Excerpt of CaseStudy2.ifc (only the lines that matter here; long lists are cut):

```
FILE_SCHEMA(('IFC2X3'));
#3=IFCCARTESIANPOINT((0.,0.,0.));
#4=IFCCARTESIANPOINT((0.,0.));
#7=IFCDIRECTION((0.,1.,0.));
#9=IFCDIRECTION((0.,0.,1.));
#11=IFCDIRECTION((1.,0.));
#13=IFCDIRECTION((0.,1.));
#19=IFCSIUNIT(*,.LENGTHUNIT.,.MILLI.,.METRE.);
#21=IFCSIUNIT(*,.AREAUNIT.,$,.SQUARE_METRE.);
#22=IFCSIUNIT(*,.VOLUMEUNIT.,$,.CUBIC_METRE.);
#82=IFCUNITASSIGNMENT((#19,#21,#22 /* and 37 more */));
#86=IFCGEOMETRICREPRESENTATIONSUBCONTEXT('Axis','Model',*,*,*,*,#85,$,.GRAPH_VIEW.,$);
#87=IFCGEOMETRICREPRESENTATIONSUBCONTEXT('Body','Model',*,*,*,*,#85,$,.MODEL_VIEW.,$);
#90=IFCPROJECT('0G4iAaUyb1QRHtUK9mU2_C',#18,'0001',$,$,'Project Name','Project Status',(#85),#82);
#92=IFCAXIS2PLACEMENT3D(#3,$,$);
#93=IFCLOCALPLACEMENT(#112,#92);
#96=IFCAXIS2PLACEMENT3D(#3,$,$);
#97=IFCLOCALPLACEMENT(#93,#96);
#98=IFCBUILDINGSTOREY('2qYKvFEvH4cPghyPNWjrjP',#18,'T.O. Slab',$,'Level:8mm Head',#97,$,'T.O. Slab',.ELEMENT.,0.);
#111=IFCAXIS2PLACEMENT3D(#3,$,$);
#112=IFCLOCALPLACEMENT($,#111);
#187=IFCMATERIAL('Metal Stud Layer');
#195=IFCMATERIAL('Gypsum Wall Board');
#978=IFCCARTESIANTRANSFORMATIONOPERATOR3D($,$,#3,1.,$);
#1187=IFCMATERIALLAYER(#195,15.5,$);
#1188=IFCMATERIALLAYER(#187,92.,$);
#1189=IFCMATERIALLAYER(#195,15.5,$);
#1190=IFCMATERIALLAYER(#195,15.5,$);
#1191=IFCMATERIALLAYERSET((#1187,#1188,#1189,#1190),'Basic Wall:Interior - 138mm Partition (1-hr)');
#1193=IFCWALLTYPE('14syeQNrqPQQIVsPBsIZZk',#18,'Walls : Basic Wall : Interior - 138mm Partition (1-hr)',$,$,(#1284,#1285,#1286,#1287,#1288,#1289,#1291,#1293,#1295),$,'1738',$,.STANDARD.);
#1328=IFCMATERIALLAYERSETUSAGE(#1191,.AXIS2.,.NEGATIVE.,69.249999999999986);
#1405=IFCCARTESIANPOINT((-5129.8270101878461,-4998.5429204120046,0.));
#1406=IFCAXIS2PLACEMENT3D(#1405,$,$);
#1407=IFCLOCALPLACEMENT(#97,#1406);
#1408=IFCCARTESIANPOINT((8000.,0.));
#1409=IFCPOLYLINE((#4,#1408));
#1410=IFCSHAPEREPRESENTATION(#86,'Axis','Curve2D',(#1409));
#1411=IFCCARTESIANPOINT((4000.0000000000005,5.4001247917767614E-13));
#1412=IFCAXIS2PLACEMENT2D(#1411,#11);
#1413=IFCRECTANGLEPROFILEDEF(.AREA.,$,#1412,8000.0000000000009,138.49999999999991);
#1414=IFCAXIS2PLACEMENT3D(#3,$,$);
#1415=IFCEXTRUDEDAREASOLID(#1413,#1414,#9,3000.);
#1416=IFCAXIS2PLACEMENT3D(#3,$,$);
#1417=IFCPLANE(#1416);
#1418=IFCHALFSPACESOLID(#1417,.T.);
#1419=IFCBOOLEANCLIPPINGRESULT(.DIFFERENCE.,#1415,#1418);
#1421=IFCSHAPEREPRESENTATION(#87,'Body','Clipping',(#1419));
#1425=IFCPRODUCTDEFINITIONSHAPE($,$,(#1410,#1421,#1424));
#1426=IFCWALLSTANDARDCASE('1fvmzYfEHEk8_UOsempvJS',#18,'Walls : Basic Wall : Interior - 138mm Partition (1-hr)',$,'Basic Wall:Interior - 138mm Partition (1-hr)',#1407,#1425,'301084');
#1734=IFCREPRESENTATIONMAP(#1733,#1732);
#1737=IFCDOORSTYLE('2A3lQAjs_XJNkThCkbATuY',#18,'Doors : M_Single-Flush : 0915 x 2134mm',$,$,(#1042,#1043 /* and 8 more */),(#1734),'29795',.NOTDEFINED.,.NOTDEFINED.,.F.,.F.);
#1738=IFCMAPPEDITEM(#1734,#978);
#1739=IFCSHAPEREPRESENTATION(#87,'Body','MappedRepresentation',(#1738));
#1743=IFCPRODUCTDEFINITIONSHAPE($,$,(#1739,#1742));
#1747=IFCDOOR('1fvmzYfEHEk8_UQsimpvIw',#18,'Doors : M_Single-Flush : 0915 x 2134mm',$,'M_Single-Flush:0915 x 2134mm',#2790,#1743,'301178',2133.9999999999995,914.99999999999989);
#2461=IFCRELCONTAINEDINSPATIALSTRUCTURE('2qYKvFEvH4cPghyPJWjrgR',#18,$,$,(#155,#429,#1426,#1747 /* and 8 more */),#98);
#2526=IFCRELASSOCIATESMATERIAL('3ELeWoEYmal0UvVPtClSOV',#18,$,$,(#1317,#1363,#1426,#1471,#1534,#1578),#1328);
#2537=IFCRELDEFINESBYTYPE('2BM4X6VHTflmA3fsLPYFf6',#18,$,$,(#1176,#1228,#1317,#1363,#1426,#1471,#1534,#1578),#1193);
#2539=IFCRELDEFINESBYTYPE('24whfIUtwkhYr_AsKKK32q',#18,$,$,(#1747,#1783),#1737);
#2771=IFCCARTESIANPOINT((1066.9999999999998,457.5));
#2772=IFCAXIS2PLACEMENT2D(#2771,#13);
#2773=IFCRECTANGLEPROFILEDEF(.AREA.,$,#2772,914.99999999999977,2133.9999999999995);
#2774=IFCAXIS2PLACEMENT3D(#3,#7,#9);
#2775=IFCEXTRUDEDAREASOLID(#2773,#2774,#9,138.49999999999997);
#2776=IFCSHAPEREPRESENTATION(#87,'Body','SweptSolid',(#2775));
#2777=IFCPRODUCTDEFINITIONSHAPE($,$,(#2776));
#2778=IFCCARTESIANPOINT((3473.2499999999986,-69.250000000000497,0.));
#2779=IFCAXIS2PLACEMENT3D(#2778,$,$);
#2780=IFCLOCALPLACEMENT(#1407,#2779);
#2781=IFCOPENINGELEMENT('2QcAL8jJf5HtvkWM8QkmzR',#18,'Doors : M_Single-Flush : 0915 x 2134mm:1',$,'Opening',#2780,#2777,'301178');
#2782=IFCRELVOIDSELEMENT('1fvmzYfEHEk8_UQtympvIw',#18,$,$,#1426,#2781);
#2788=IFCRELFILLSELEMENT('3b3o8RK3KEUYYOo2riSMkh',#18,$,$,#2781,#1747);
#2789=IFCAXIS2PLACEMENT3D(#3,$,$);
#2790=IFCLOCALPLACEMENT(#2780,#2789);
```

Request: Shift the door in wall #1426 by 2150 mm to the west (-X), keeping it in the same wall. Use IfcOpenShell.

```python
import ifcopenshell
import ifcopenshell.api.geometry
import ifcopenshell.util.placement
import ifcopenshell.util.unit

model = ifcopenshell.open("CaseStudy2.ifc")
unit_scale = ifcopenshell.util.unit.calculate_unit_scale(model)

door = model.by_guid("1fvmzYfEHEk8_UQsimpvIw")
opening = door.FillsVoids[0].RelatingOpeningElement
wall = opening.VoidsElements[0].RelatingBuildingElement

wall_matrix = ifcopenshell.util.placement.get_local_placement(wall.ObjectPlacement)
shift = wall_matrix[:3, 0] * -2.15 / unit_scale
before = ifcopenshell.util.placement.get_local_placement(door.ObjectPlacement)[:3, 3].copy()

# The door is placed relative to its opening, so it follows when the opening moves.
matrix = ifcopenshell.util.placement.get_local_placement(opening.ObjectPlacement)
matrix[:3, 3] += shift
ifcopenshell.api.geometry.edit_object_placement(
    model, product=opening, matrix=matrix, is_si=False, should_transform_children=True
)

after = ifcopenshell.util.placement.get_local_placement(door.ObjectPlacement)[:3, 3]
print("door moved by", (after - before).round(3) + 0.0)

model.write("CaseStudy2_rev.ifc")
```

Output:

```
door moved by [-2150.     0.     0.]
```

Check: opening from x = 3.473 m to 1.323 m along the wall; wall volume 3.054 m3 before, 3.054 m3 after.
